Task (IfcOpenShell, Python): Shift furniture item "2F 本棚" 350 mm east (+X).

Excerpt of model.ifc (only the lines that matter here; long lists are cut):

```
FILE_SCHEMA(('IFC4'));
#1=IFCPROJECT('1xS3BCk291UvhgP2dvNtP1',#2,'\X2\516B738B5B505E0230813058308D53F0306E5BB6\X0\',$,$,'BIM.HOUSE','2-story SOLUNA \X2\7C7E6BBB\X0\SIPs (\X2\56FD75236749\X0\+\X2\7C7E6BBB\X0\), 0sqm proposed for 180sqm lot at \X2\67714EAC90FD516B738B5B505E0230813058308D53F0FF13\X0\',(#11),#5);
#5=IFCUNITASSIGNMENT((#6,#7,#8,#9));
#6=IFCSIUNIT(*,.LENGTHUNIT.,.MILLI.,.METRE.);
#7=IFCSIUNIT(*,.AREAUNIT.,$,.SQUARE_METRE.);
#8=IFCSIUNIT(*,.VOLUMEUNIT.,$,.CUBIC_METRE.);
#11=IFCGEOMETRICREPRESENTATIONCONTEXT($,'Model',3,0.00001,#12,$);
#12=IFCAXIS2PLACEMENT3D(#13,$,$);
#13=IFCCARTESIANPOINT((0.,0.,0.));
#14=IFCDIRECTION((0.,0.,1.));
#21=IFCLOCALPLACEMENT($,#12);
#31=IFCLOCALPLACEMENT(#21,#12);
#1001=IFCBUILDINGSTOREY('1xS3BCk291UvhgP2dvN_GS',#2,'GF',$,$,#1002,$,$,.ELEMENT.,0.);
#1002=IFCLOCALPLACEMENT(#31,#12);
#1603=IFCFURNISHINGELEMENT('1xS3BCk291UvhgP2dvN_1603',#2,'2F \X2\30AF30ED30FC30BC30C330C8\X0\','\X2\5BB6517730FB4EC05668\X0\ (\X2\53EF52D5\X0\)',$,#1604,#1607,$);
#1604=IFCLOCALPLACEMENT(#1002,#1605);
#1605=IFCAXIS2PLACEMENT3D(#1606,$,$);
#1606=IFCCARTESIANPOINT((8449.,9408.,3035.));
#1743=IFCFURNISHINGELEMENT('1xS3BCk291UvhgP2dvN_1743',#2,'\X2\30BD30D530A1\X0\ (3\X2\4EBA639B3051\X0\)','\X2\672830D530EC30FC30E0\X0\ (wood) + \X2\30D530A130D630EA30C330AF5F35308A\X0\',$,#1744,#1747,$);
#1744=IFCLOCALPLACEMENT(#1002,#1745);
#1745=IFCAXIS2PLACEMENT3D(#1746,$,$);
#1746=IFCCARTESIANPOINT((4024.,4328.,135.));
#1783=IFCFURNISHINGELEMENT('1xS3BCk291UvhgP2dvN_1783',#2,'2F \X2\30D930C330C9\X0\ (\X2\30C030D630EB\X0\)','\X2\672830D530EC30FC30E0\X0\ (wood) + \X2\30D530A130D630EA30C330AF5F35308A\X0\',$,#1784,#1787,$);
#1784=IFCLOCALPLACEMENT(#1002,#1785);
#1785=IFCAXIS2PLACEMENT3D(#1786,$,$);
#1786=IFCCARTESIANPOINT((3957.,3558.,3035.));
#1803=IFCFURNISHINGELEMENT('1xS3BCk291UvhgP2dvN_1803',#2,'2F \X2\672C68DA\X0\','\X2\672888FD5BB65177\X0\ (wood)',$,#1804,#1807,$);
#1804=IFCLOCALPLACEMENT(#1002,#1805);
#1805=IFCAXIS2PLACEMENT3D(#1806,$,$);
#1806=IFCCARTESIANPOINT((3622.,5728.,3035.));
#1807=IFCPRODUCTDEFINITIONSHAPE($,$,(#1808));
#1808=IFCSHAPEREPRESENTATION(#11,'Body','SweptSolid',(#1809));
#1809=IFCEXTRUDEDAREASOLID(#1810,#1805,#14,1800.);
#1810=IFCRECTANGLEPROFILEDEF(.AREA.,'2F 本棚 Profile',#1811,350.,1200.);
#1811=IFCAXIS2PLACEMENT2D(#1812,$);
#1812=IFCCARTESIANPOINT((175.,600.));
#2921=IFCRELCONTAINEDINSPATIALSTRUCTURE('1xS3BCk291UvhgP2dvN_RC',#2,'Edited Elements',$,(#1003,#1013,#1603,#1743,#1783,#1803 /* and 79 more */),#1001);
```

```python
import ifcopenshell
import ifcopenshell.api.geometry
import ifcopenshell.util.placement
import ifcopenshell.util.unit

model = ifcopenshell.open("model.ifc")
unit_scale = ifcopenshell.util.unit.calculate_unit_scale(model)

item = model.by_guid("1xS3BCk291UvhgP2dvN_1803")
matrix = ifcopenshell.util.placement.get_local_placement(item.ObjectPlacement)
matrix[0, 3] += 0.35 / unit_scale
ifcopenshell.api.geometry.edit_object_placement(model, product=item, matrix=matrix, is_si=False)

print(ifcopenshell.util.placement.get_local_placement(item.ObjectPlacement).round(3) + 0.0)

model.write("model_rev.ifc")
```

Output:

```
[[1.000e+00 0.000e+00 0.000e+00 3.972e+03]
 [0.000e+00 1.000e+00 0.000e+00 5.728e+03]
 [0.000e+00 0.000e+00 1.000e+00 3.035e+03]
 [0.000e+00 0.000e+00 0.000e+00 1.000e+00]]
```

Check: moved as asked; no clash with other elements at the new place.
